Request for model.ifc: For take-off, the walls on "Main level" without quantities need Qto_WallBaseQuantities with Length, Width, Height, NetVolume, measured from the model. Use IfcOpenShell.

First a look at what the model holds.

```python
import ifcopenshell
import ifcopenshell.util.element
import ifcopenshell.util.unit

model = ifcopenshell.open("model.ifc")
print(model.schema)
for unit_type in ("LENGTHUNIT", "AREAUNIT", "VOLUMEUNIT"):
    print(unit_type, ifcopenshell.util.unit.calculate_unit_scale(model, unit_type))
storey = next(s for s in model.by_type("IfcBuildingStorey") if s.Name == "Main level")
walls = [e for e in ifcopenshell.util.element.get_decomposition(storey) if e.is_a("IfcWall")]
for e in sorted(walls, key=lambda e: e.id()):
    print(e.id(), e.is_a(), e.Name, list(ifcopenshell.util.element.get_psets(e, qtos_only=True)), sep=" | ")
```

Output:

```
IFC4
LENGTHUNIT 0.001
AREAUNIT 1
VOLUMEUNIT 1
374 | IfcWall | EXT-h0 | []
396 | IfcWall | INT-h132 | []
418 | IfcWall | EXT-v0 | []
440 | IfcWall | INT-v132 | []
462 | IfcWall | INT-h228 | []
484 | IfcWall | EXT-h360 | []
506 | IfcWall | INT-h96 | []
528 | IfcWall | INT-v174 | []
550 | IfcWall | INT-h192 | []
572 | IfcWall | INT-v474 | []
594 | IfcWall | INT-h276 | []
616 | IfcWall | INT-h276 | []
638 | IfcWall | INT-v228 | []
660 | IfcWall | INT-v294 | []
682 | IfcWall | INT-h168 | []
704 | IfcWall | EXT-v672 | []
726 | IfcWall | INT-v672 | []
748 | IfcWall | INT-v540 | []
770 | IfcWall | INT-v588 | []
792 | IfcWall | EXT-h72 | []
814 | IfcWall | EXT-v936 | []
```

```python
import ifcopenshell
import ifcopenshell.api.pset
import ifcopenshell.geom
import ifcopenshell.util.element
import ifcopenshell.util.shape
import ifcopenshell.util.unit

model = ifcopenshell.open("model.ifc")
unit_scale = ifcopenshell.util.unit.calculate_unit_scale(model)
volume_scale = ifcopenshell.util.unit.calculate_unit_scale(model, "VOLUMEUNIT")
settings = ifcopenshell.geom.settings()

storey = next(s for s in model.by_type("IfcBuildingStorey") if s.Name == "Main level")
walls = [e for e in ifcopenshell.util.element.get_decomposition(storey) if e.is_a("IfcWall")]

for e in sorted(walls, key=lambda e: e.id()):
    if ifcopenshell.util.element.get_psets(e, qtos_only=True, should_inherit=False):
        continue
    # Geometry comes back in metres, in the element's own axes.
    shape = ifcopenshell.geom.create_shape(settings, e)
    values = {
        "Length": ifcopenshell.util.shape.get_x(shape.geometry) / unit_scale,
        "Width": ifcopenshell.util.shape.get_y(shape.geometry) / unit_scale,
        "Height": ifcopenshell.util.shape.get_z(shape.geometry) / unit_scale,
        "NetVolume": ifcopenshell.util.shape.get_volume(shape.geometry) / volume_scale,
    }
    qto = ifcopenshell.api.pset.add_qto(model, product=e, name="Qto_WallBaseQuantities")
    ifcopenshell.api.pset.edit_qto(model, qto=qto, properties=values)
    print(e.id(), {k: round(v, 3) for k, v in values.items()})

model.write("model_rev.ifc")
```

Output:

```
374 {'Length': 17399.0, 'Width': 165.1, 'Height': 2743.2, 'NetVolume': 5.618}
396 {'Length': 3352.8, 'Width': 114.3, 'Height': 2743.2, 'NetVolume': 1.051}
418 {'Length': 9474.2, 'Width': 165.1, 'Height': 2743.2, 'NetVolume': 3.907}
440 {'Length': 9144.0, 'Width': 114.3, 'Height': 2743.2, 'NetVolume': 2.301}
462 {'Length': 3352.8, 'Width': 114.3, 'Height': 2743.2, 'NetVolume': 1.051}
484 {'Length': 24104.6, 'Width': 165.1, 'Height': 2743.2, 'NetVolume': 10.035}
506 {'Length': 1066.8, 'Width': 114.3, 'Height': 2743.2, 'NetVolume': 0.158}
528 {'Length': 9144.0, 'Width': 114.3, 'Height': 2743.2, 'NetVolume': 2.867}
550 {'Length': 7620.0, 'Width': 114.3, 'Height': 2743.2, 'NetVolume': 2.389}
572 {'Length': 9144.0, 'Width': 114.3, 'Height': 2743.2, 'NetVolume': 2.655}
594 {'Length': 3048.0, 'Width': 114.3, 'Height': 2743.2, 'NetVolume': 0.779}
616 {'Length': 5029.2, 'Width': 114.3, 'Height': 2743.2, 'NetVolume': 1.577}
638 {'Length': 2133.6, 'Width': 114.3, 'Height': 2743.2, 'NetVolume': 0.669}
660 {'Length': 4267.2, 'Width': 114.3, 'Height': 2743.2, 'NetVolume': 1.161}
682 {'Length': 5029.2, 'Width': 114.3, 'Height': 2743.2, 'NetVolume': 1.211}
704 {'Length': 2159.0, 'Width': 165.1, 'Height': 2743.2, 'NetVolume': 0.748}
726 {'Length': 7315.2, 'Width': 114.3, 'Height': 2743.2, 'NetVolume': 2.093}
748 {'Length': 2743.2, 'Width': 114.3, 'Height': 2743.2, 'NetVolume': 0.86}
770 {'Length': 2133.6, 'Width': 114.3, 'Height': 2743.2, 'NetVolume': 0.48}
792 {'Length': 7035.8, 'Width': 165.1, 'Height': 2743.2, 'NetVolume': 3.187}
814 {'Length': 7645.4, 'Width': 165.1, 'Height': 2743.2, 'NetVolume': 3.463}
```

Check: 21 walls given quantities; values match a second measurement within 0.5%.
